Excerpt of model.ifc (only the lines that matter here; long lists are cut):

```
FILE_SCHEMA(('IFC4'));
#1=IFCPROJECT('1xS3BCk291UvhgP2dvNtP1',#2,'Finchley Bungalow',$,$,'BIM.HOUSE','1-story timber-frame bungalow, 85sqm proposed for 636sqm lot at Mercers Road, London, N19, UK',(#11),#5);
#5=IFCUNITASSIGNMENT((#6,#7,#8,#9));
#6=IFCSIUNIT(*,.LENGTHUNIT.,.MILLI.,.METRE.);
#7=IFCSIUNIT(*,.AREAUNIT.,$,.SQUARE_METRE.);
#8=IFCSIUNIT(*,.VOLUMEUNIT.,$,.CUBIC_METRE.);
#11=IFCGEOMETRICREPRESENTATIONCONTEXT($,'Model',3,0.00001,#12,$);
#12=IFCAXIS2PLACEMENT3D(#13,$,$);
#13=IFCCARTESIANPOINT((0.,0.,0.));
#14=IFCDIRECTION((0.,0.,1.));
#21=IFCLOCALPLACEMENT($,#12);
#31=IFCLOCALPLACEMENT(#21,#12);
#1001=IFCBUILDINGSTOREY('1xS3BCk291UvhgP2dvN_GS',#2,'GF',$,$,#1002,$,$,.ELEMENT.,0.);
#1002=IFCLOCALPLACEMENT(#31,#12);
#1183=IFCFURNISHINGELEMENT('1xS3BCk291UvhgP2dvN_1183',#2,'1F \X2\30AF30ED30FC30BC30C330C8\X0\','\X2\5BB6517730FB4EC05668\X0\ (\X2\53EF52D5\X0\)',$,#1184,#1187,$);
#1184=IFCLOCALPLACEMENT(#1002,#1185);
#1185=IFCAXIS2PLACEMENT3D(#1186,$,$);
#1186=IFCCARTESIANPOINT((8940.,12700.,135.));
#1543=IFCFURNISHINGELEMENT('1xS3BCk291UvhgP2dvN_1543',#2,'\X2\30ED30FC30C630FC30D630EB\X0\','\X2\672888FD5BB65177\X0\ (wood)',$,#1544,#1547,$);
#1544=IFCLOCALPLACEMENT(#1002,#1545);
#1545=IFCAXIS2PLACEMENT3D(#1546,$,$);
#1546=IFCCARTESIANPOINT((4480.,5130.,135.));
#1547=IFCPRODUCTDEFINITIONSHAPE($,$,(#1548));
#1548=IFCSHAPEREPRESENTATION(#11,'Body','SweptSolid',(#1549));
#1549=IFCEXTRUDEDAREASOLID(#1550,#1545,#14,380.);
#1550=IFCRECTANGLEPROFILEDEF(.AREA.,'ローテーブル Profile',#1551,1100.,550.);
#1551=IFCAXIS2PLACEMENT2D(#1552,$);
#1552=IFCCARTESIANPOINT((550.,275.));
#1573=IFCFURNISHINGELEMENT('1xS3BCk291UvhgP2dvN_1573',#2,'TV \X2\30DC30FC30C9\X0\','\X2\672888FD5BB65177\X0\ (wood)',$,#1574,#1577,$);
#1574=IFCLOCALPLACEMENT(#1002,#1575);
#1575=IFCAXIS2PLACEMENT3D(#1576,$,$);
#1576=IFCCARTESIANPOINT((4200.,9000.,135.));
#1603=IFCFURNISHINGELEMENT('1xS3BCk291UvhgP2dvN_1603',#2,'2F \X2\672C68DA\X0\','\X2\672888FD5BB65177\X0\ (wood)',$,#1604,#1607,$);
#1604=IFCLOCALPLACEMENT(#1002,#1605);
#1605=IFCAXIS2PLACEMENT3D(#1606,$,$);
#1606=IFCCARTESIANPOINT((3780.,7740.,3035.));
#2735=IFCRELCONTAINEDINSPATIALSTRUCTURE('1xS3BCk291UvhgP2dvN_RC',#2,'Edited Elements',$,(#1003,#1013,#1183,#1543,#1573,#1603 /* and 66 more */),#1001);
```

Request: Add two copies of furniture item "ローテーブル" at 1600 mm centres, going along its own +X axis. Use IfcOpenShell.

```python
import ifcopenshell
import ifcopenshell.api.geometry
import ifcopenshell.api.root
import ifcopenshell.util.element
import ifcopenshell.util.placement
import ifcopenshell.util.unit

model = ifcopenshell.open("model.ifc")
unit_scale = ifcopenshell.util.unit.calculate_unit_scale(model)


def reuse_history(source, copy):
    """copy_class also copies each property set's owner history, people and application; keep the originals."""
    for rel in copy.IsDefinedBy:
        if rel.is_a("IfcRelDefinesByProperties") and (history := rel.RelatingPropertyDefinition.OwnerHistory):
            rel.RelatingPropertyDefinition.OwnerHistory = source.OwnerHistory
            ifcopenshell.util.element.remove_deep2(model, history)


source = model.by_id(1543)
base = ifcopenshell.util.placement.get_local_placement(source.ObjectPlacement)
step = base[:3, 0] * 1.6 / unit_scale

for i in range(1, 3):
    copy = ifcopenshell.api.root.copy_class(model, product=source)
    copy.Representation = ifcopenshell.util.element.copy_deep(
        model, source.Representation, exclude=["IfcGeometricRepresentationContext", "IfcRepresentationMap"]
    )
    reuse_history(source, copy)
    matrix = base.copy()
    matrix[:3, 3] += i * step
    print("added at", matrix[:3, 3].round(3) + 0.0)
    ifcopenshell.api.geometry.edit_object_placement(model, product=copy, matrix=matrix, is_si=False)

model.write("model_rev.ifc")
```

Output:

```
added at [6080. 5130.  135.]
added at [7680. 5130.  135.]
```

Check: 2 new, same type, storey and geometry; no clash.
